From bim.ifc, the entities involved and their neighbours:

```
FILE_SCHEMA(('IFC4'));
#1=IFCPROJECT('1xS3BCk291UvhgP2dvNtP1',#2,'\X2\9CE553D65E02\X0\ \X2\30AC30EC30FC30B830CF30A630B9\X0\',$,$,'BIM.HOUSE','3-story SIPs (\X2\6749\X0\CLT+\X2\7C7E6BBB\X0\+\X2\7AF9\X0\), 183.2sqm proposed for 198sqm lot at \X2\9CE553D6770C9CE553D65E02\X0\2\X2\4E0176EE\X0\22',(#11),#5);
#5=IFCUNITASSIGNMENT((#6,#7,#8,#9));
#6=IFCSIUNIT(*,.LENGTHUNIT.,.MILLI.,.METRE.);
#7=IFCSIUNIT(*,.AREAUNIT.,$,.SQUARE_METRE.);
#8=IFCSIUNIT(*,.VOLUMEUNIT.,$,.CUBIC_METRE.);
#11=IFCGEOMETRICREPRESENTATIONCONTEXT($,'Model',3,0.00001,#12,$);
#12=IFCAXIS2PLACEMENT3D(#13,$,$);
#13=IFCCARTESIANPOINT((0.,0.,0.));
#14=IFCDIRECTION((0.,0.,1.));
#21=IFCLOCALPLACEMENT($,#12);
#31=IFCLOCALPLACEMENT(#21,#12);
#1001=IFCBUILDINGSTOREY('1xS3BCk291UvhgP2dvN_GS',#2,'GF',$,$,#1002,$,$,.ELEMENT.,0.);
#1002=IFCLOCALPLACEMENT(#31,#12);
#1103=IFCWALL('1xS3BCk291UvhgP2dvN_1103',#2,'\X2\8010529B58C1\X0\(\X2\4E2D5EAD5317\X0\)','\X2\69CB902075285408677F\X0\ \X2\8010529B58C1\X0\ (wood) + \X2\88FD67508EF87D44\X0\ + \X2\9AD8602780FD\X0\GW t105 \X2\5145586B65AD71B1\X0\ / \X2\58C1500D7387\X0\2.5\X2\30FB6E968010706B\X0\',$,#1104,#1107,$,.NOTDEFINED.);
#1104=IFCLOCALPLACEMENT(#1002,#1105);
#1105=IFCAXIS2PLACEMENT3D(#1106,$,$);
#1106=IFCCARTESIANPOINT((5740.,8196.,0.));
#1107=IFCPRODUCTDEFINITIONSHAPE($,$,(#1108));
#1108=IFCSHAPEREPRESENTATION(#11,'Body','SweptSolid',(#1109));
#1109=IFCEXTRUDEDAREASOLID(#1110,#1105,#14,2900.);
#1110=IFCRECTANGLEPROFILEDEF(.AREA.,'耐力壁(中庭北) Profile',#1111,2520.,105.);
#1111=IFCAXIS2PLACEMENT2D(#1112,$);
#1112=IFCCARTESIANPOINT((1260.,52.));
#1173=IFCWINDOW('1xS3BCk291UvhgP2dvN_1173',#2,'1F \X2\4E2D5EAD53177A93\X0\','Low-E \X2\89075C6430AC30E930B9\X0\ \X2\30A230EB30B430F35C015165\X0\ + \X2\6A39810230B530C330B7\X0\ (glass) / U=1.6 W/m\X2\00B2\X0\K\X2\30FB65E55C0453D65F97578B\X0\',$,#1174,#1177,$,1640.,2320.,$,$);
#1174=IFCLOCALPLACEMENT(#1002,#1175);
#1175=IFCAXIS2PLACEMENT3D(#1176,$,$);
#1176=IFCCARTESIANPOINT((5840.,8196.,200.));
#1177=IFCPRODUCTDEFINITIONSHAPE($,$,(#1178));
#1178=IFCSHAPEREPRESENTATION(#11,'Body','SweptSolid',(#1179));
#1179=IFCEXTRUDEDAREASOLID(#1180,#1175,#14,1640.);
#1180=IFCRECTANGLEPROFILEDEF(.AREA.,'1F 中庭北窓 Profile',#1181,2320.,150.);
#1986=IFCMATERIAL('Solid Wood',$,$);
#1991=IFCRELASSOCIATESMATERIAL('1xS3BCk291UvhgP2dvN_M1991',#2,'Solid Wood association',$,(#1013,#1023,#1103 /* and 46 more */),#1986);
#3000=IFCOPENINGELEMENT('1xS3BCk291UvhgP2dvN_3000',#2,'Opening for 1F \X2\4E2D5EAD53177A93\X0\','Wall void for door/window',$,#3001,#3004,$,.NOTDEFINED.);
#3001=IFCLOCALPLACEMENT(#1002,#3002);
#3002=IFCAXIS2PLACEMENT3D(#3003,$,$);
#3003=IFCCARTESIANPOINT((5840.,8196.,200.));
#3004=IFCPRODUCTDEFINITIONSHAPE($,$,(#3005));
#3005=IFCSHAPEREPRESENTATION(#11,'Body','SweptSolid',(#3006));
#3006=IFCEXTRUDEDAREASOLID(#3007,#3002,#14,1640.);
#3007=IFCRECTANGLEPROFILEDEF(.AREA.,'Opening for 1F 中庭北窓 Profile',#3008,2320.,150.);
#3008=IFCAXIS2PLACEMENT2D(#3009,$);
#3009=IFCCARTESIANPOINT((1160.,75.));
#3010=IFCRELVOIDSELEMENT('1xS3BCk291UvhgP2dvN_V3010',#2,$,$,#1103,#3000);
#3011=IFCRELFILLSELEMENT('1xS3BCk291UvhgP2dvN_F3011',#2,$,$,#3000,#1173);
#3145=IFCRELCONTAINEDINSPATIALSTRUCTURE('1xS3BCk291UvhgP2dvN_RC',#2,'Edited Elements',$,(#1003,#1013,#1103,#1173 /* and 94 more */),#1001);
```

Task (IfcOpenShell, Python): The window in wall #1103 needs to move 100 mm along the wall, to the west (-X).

```python
import ifcopenshell
import ifcopenshell.api.geometry
import ifcopenshell.util.placement

model = ifcopenshell.open("bim.ifc")

window = model.by_guid("1xS3BCk291UvhgP2dvN_1173")
opening = window.FillsVoids[0].RelatingOpeningElement
wall = opening.VoidsElements[0].RelatingBuildingElement

wall_matrix = ifcopenshell.util.placement.get_local_placement(wall.ObjectPlacement)
shift = wall_matrix[:3, 0] * -100.0
before = ifcopenshell.util.placement.get_local_placement(window.ObjectPlacement)[:3, 3].copy()

# The window is not placed relative to its opening, so move both.
for product in (opening, window):
    matrix = ifcopenshell.util.placement.get_local_placement(product.ObjectPlacement)
    matrix[:3, 3] += shift
    ifcopenshell.api.geometry.edit_object_placement(model, product=product, matrix=matrix, is_si=False)

after = ifcopenshell.util.placement.get_local_placement(window.ObjectPlacement)[:3, 3]
print("window moved by", (after - before).round(3) + 0.0)

model.write("bim_rev.ifc")
```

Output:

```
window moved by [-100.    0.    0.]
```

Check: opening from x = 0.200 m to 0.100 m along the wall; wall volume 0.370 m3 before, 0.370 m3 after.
